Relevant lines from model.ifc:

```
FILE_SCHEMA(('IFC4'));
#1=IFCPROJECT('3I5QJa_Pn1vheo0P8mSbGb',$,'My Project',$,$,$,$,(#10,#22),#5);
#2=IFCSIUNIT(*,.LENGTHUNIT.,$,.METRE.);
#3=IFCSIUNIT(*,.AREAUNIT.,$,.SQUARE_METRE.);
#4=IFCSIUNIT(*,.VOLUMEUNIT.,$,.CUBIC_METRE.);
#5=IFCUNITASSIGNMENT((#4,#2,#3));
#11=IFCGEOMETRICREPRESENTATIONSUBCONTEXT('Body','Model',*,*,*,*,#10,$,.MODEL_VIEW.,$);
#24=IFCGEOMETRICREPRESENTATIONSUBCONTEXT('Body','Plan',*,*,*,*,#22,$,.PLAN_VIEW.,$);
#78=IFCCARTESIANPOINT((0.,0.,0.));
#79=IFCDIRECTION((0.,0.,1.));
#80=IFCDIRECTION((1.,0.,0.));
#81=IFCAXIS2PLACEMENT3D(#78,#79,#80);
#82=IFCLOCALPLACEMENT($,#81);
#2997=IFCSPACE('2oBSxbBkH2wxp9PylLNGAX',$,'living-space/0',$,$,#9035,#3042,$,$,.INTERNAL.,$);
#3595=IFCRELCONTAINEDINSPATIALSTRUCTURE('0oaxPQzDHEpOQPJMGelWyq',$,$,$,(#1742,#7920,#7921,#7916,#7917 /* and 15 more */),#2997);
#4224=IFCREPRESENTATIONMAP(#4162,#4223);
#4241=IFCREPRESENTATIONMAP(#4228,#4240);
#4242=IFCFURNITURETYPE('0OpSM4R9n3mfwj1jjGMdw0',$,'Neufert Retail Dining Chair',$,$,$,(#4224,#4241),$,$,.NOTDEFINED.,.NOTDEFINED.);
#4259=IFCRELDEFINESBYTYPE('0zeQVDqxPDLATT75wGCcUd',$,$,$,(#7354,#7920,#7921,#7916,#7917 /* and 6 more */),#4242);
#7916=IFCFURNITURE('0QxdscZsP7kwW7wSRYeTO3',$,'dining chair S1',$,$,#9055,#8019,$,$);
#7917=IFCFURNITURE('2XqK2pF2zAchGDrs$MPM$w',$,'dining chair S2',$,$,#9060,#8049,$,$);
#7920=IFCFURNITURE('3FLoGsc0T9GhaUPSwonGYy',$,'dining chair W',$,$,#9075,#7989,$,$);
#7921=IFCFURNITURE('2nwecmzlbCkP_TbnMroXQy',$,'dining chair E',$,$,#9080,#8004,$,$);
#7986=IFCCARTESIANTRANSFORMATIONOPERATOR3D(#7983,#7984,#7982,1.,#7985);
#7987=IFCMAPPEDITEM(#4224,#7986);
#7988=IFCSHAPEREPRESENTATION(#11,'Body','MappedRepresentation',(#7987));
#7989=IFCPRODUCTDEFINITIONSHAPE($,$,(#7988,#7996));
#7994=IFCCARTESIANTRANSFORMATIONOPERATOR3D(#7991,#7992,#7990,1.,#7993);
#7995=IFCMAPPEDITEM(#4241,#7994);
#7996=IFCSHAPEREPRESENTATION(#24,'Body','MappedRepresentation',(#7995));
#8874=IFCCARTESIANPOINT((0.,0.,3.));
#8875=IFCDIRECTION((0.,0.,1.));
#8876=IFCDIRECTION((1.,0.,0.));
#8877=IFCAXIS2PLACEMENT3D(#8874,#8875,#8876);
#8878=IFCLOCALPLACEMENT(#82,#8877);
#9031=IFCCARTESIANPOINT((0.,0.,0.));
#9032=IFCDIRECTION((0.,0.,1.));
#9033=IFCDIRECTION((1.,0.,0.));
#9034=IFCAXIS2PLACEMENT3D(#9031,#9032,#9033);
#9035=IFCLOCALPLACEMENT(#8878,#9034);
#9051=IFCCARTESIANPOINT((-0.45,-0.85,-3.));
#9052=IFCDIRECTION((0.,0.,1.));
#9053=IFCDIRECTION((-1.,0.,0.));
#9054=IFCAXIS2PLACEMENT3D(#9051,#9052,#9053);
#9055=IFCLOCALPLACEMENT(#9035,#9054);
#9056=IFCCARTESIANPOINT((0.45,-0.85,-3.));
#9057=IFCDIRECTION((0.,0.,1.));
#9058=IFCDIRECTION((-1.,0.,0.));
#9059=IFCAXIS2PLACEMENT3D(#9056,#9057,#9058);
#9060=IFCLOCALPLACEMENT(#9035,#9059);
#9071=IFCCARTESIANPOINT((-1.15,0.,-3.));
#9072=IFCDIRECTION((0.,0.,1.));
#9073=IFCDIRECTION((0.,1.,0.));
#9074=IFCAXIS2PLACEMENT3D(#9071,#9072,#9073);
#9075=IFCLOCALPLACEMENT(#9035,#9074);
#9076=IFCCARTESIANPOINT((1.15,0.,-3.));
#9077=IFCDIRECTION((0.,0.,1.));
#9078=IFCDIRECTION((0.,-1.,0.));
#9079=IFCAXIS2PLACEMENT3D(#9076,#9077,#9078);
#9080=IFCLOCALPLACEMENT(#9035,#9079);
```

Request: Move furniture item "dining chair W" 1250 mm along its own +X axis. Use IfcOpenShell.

```python
import ifcopenshell
import ifcopenshell.api.geometry
import ifcopenshell.util.placement
import ifcopenshell.util.unit

model = ifcopenshell.open("model.ifc")
unit_scale = ifcopenshell.util.unit.calculate_unit_scale(model)

item = model.by_guid("3FLoGsc0T9GhaUPSwonGYy")
matrix = ifcopenshell.util.placement.get_local_placement(item.ObjectPlacement)
matrix[:3, 3] += matrix[:3, 0] * 1.25 / unit_scale
ifcopenshell.api.geometry.edit_object_placement(model, product=item, matrix=matrix, is_si=False)

print(ifcopenshell.util.placement.get_local_placement(item.ObjectPlacement).round(3) + 0.0)

model.write("model_updated.ifc")
```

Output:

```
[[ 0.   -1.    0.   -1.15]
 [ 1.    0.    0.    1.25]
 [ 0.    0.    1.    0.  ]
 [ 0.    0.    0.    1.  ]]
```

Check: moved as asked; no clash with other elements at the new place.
